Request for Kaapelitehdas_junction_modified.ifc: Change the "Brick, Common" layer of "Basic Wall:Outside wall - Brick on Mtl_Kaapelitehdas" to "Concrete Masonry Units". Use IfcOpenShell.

First a look at what the model holds.

```python
import ifcopenshell
import ifcopenshell.util.element

model = ifcopenshell.open("Kaapelitehdas_junction_modified.ifc")
print(model.schema)
for layer_set in model.by_type("IfcMaterialLayerSet"):
    if layer_set.LayerSetName == "Basic Wall:Outside wall - Brick on Mtl_Kaapelitehdas":
        for layer in layer_set.MaterialLayers:
            print(layer.id(), layer.Material and layer.Material.Name, layer.LayerThickness, sep=" | ")
        print(len(ifcopenshell.util.element.get_elements_by_material(model, layer_set)), "elements and types use it")
print(sorted(m.Name for m in model.by_type("IfcMaterial") if m.Name)[:60])
```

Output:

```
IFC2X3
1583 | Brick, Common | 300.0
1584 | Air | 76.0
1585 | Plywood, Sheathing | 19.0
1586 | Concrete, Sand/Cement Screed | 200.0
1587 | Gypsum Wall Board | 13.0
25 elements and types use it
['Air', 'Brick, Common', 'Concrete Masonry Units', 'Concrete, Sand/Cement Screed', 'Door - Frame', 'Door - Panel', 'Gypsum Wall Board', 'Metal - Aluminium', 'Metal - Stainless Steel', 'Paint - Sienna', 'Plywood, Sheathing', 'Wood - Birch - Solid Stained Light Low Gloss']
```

```python
import ifcopenshell
import ifcopenshell.api.material

model = ifcopenshell.open("Kaapelitehdas_junction_modified.ifc")

layer_set = next(s for s in model.by_type("IfcMaterialLayerSet") if s.LayerSetName == "Basic Wall:Outside wall - Brick on Mtl_Kaapelitehdas")
layer = next(l for l in layer_set.MaterialLayers if l.Material and l.Material.Name == "Brick, Common")
material = next(m for m in model.by_type("IfcMaterial") if m.Name == "Concrete Masonry Units")

# Point this one layer at the other material; renaming the old one would change it everywhere.
ifcopenshell.api.material.edit_layer(model, layer=layer, attributes={}, material=material)

print([l.Material.Name if l.Material else None for l in layer_set.MaterialLayers])

model.write("Kaapelitehdas_junction_modified_v2.ifc")
```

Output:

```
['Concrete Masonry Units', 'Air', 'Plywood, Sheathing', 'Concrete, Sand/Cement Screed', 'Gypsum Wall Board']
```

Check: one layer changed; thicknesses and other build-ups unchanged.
